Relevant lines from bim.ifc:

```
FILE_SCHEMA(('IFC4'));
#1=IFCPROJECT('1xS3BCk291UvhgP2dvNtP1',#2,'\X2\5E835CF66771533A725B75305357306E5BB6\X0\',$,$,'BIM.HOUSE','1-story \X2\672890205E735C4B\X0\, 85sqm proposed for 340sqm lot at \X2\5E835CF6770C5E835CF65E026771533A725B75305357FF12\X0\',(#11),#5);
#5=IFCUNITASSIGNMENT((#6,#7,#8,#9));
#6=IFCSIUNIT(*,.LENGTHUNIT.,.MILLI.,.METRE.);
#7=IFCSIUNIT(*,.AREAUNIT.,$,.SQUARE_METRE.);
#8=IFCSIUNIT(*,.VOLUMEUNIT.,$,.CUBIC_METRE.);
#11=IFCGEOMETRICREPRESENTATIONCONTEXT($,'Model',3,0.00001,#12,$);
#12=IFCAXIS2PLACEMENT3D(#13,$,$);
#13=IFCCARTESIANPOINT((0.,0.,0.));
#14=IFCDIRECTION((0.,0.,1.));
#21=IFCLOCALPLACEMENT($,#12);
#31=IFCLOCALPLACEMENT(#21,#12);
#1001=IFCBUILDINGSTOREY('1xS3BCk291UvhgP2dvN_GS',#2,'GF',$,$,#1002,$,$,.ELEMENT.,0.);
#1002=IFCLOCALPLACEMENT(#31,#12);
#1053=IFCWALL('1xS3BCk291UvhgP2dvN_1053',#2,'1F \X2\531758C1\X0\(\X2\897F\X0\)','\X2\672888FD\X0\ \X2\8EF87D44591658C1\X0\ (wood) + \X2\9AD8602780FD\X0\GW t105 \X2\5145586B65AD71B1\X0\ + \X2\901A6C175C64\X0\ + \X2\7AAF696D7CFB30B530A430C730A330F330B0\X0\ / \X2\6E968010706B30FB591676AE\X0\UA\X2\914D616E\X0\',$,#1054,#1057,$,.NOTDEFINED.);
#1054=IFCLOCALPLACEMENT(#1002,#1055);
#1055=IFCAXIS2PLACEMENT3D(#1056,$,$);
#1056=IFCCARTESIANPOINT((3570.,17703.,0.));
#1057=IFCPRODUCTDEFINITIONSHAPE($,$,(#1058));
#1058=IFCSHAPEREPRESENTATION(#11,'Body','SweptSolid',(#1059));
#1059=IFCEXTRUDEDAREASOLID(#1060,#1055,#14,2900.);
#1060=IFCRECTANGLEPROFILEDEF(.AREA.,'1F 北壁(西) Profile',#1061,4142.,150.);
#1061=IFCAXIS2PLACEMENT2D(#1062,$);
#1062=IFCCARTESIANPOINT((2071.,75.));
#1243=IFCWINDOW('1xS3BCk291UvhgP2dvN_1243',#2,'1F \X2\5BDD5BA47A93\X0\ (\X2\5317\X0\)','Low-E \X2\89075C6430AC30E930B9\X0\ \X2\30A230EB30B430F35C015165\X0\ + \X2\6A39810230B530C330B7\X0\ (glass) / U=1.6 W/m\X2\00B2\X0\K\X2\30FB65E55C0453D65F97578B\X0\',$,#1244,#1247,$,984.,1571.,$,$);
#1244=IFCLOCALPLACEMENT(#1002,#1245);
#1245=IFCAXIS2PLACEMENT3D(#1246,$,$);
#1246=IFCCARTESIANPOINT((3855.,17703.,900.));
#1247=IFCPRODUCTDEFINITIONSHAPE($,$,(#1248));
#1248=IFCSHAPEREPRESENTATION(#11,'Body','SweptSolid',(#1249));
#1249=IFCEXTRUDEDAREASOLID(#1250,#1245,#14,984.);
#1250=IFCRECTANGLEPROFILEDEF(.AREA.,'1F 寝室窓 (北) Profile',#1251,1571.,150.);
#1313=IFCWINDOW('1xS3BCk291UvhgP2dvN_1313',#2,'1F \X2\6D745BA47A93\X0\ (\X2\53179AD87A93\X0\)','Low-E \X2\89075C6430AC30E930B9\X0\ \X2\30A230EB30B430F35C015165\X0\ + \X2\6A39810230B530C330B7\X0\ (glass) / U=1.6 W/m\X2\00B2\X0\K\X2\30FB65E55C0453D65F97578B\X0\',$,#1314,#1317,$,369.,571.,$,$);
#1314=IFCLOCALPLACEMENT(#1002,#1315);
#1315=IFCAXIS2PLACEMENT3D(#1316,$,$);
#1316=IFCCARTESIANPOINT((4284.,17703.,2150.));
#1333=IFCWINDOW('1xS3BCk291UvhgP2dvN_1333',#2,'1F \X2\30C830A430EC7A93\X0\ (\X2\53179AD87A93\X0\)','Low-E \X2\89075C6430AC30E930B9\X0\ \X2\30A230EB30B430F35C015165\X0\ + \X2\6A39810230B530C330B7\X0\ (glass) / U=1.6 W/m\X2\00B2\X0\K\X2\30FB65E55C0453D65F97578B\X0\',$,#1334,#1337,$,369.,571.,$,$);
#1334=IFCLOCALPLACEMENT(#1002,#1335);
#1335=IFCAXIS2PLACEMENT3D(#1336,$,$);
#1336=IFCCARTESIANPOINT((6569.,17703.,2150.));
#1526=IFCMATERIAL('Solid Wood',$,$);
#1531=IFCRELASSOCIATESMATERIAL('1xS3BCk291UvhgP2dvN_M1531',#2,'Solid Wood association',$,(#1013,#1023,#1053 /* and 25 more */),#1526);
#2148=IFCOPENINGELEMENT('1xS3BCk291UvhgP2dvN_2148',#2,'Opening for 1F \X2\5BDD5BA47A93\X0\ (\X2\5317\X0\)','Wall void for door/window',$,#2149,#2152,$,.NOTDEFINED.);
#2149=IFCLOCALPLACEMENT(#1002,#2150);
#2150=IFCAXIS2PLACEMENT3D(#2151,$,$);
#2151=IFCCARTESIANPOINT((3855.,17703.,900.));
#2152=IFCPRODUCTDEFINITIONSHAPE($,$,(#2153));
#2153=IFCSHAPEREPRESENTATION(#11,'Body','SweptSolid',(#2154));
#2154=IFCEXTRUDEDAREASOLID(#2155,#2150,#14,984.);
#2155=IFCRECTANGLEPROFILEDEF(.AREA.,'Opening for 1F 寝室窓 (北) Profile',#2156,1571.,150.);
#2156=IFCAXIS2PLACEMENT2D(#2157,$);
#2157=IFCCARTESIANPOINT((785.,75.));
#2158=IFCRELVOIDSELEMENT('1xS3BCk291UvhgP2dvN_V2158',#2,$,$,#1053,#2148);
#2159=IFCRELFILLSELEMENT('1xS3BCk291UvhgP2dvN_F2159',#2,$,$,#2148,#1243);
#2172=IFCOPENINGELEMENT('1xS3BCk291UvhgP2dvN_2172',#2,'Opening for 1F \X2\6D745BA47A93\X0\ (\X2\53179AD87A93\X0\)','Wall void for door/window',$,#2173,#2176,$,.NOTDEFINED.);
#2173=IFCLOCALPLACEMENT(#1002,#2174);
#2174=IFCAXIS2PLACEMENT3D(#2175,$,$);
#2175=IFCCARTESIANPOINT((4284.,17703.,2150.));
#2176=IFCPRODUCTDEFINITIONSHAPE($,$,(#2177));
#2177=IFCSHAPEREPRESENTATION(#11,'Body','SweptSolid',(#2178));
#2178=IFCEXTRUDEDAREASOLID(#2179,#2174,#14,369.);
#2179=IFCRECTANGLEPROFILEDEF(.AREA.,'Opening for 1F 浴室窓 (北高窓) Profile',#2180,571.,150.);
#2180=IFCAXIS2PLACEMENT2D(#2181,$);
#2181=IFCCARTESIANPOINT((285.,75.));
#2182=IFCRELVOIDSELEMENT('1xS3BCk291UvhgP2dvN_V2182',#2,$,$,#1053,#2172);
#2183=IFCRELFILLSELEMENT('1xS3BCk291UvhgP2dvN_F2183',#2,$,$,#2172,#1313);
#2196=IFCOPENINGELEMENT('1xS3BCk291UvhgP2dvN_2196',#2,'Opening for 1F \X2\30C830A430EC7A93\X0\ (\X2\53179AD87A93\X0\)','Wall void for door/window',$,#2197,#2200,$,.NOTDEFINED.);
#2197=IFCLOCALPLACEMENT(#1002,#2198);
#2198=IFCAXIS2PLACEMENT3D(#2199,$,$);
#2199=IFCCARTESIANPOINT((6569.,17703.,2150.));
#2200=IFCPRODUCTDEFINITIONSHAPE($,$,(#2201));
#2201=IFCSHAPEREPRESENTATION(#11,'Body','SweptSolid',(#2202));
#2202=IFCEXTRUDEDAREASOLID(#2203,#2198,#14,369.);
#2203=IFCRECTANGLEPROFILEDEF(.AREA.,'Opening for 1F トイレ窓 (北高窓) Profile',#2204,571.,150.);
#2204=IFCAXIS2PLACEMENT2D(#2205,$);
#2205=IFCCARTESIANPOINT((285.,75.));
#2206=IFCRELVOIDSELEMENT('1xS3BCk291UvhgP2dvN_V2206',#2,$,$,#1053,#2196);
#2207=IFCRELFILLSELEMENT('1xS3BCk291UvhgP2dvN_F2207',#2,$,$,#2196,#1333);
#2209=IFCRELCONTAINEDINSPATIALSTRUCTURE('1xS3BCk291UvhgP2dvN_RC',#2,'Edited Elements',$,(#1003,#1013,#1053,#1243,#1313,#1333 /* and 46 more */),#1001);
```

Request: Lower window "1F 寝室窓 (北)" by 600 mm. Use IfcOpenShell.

```python
import numpy as np
import ifcopenshell
import ifcopenshell.api.geometry
import ifcopenshell.util.placement
import ifcopenshell.util.unit

model = ifcopenshell.open("bim.ifc")
unit_scale = ifcopenshell.util.unit.calculate_unit_scale(model)

window = model.by_id(1243)
opening = window.FillsVoids[0].RelatingOpeningElement
dz = -0.6 / unit_scale

shift = np.array([0.0, 0.0, dz])
# The window is not placed relative to its opening, so move both.
for product in (opening, window):
    matrix = ifcopenshell.util.placement.get_local_placement(product.ObjectPlacement)
    matrix[:3, 3] += shift
    ifcopenshell.api.geometry.edit_object_placement(model, product=product, matrix=matrix, is_si=False)

print(f"moved by {dz * unit_scale:+.3f} m")

model.write("bim_rev.ifc")
```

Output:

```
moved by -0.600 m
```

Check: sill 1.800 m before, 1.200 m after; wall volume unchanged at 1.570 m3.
